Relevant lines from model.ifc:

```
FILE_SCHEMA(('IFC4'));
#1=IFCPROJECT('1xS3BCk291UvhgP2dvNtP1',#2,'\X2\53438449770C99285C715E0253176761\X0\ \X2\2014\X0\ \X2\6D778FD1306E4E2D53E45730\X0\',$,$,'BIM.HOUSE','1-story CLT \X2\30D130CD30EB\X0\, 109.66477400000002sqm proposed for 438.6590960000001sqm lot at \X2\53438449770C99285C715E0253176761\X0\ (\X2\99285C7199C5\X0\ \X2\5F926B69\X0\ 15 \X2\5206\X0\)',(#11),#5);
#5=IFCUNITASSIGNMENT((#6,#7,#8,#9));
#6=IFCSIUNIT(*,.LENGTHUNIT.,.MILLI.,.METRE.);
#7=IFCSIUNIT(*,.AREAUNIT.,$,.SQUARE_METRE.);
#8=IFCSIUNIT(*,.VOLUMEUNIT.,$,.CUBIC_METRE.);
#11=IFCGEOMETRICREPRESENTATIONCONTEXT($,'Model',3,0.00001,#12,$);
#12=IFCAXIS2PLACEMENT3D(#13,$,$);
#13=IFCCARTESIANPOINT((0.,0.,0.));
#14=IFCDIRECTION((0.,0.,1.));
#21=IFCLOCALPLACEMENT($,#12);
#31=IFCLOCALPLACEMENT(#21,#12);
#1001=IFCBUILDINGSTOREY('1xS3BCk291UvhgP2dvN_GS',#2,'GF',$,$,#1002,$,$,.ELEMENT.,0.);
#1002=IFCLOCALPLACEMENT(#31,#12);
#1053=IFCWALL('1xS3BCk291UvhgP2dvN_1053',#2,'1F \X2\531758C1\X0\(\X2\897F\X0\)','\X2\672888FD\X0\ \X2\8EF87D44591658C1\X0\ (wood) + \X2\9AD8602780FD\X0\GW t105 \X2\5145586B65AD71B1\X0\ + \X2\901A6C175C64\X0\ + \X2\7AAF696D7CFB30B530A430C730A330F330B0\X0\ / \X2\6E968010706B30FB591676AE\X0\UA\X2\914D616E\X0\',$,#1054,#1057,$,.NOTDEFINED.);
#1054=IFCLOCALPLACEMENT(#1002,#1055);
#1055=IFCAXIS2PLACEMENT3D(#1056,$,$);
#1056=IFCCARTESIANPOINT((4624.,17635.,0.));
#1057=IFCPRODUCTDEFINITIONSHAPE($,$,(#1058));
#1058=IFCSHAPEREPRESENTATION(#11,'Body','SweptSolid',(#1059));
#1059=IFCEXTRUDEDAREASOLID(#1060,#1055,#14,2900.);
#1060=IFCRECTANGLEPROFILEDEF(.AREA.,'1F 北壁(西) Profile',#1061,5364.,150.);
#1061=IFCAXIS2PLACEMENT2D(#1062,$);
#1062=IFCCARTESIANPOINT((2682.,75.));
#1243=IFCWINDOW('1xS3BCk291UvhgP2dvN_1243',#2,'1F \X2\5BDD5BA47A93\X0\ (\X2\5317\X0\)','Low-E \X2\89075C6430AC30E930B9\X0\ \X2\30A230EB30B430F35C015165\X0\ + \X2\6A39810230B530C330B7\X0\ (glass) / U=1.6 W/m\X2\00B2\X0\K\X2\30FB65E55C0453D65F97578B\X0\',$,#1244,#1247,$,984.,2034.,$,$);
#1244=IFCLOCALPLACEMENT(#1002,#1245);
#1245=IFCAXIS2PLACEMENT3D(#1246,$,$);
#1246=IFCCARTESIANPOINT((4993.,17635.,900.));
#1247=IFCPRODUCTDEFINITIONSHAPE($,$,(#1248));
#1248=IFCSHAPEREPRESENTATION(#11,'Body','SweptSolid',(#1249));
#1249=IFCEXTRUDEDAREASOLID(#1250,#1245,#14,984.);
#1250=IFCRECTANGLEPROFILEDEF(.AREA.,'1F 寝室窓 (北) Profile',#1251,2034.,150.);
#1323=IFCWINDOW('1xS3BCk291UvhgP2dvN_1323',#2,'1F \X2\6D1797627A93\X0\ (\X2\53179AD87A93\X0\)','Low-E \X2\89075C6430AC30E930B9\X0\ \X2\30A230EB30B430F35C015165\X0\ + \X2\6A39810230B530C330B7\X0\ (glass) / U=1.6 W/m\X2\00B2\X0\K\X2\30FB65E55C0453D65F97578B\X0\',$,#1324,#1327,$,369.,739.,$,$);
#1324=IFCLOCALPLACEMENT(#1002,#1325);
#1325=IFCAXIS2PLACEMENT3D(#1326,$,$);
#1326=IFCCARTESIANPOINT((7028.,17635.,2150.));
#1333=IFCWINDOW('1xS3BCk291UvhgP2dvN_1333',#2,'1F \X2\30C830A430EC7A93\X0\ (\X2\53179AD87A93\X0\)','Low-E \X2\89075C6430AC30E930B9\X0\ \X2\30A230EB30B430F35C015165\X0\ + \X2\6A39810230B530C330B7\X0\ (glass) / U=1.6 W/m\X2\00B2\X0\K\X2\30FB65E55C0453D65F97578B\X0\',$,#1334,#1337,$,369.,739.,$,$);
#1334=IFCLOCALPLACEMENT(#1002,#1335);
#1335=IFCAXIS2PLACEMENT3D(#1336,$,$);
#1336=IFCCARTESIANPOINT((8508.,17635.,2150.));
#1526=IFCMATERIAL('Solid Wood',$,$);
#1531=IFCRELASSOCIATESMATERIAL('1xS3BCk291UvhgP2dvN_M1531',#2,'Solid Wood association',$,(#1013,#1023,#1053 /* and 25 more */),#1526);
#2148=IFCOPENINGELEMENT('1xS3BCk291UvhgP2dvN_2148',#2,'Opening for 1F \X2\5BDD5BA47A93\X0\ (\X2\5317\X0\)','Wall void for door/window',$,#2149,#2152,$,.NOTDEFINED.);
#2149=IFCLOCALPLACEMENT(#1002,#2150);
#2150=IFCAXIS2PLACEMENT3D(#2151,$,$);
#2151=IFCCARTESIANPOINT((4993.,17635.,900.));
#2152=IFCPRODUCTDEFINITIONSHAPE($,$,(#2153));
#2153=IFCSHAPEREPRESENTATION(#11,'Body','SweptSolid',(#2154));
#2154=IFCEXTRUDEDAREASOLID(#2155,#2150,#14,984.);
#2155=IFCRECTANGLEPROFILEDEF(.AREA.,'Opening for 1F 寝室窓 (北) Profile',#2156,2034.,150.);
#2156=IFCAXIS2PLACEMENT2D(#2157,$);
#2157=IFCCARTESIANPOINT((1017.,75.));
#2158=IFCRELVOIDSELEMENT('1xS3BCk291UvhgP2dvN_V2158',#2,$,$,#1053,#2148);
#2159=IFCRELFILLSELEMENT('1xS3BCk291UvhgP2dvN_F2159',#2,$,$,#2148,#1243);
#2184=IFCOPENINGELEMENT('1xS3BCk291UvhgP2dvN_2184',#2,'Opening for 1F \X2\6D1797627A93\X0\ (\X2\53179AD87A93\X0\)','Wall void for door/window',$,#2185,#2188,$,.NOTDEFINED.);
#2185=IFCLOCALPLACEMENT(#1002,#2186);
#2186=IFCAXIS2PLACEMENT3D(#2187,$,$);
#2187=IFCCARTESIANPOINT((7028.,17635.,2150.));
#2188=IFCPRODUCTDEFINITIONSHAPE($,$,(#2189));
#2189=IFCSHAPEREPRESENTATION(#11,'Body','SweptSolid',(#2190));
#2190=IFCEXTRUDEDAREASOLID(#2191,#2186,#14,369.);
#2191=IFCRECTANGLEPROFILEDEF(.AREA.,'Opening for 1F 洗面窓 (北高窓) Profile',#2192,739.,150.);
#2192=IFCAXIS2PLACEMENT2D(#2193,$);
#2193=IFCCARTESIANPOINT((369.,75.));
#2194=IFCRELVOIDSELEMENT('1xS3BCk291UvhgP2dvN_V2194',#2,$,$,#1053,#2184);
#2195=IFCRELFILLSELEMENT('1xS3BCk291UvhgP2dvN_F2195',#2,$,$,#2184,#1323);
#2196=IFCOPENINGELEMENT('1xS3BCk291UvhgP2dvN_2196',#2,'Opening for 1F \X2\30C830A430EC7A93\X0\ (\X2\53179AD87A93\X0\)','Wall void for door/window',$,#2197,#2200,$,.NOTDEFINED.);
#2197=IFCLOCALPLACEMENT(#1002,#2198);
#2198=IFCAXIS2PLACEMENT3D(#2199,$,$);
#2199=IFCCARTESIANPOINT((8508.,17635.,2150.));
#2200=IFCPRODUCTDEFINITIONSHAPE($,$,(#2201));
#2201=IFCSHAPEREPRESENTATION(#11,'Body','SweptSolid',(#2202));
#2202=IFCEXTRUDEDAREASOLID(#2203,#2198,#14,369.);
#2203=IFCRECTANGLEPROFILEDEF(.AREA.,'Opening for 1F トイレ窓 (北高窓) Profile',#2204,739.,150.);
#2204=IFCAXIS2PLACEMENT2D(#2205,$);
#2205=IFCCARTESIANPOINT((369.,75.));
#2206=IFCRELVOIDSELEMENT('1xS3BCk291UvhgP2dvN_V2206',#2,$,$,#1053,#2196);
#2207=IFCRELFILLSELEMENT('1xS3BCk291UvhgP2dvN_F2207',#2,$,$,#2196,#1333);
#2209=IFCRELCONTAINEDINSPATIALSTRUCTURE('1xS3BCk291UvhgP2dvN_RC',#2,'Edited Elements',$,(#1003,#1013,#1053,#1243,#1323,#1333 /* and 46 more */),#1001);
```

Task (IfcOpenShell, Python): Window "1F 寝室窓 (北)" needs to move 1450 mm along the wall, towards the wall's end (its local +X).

```python
import ifcopenshell
import ifcopenshell.api.geometry
import ifcopenshell.util.placement
import ifcopenshell.util.unit

model = ifcopenshell.open("model.ifc")
unit_scale = ifcopenshell.util.unit.calculate_unit_scale(model)

window = model.by_guid("1xS3BCk291UvhgP2dvN_1243")
opening = window.FillsVoids[0].RelatingOpeningElement
wall = opening.VoidsElements[0].RelatingBuildingElement

wall_matrix = ifcopenshell.util.placement.get_local_placement(wall.ObjectPlacement)
shift = wall_matrix[:3, 0] * 1.45 / unit_scale
before = ifcopenshell.util.placement.get_local_placement(window.ObjectPlacement)[:3, 3].copy()

# The window is not placed relative to its opening, so move both.
for product in (opening, window):
    matrix = ifcopenshell.util.placement.get_local_placement(product.ObjectPlacement)
    matrix[:3, 3] += shift
    ifcopenshell.api.geometry.edit_object_placement(model, product=product, matrix=matrix, is_si=False)

after = ifcopenshell.util.placement.get_local_placement(window.ObjectPlacement)[:3, 3]
print("window moved by", (after - before).round(3) + 0.0)

model.write("model_v2.ifc")
```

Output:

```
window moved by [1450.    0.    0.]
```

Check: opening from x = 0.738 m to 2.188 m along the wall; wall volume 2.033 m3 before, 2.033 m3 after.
